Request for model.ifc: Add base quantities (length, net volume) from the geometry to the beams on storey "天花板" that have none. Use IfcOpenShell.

First a look at what the model holds.

```python
import ifcopenshell
import ifcopenshell.util.element
import ifcopenshell.util.unit

model = ifcopenshell.open("model.ifc")
print(model.schema)
for unit_type in ("LENGTHUNIT", "AREAUNIT", "VOLUMEUNIT"):
    print(unit_type, ifcopenshell.util.unit.calculate_unit_scale(model, unit_type))
storey = next(s for s in model.by_type("IfcBuildingStorey") if s.Name == "天花板")
beams = [e for e in ifcopenshell.util.element.get_decomposition(storey) if e.is_a("IfcBeam")]
for e in sorted(beams, key=lambda e: e.id()):
    print(e.id(), e.is_a(), e.Name, list(ifcopenshell.util.element.get_psets(e, qtos_only=True)), sep=" | ")
```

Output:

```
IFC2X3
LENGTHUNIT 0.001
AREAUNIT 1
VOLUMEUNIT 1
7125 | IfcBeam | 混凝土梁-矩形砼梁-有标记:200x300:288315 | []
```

```python
import ifcopenshell
import ifcopenshell.api.pset
import ifcopenshell.geom
import ifcopenshell.util.element
import ifcopenshell.util.shape
import ifcopenshell.util.unit

model = ifcopenshell.open("model.ifc")
unit_scale = ifcopenshell.util.unit.calculate_unit_scale(model)
volume_scale = ifcopenshell.util.unit.calculate_unit_scale(model, "VOLUMEUNIT")
settings = ifcopenshell.geom.settings()

storey = next(s for s in model.by_type("IfcBuildingStorey") if s.Name == "天花板")
beams = [e for e in ifcopenshell.util.element.get_decomposition(storey) if e.is_a("IfcBeam")]

for e in sorted(beams, key=lambda e: e.id()):
    if ifcopenshell.util.element.get_psets(e, qtos_only=True, should_inherit=False):
        continue
    # Geometry comes back in metres, in the element's own axes.
    shape = ifcopenshell.geom.create_shape(settings, e)
    values = {
        "Length": ifcopenshell.util.shape.get_max_xyz(shape.geometry) / unit_scale,
        "NetVolume": ifcopenshell.util.shape.get_volume(shape.geometry) / volume_scale,
    }
    qto = ifcopenshell.api.pset.add_qto(model, product=e, name="BaseQuantities")
    ifcopenshell.api.pset.edit_qto(model, qto=qto, properties=values)
    print(e.id(), {k: round(v, 3) for k, v in values.items()})

model.write("model_edited.ifc")
```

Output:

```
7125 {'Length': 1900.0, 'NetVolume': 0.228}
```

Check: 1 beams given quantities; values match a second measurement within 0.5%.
